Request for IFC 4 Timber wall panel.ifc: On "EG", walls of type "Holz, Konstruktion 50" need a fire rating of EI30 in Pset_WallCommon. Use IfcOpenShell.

First a look at what the model holds.

```python
import ifcopenshell
import ifcopenshell.util.element

model = ifcopenshell.open("IFC 4 Timber wall panel.ifc")
print(model.schema)
storey = next(s for s in model.by_type("IfcBuildingStorey") if s.Name == "EG")
walls = [e for e in ifcopenshell.util.element.get_decomposition(storey) if e.is_a("IfcWall")]
seen = {}
for e in walls:
    element_type = ifcopenshell.util.element.get_type(e)
    key = (element_type.Name if element_type != e and element_type else None, ifcopenshell.util.element.get_pset(e, "Pset_WallCommon", "FireRating"))
    seen[key] = seen.get(key, 0) + 1
for (name, value), count in sorted(seen.items(), key=str):
    print(count, "x", name, "|", value)
```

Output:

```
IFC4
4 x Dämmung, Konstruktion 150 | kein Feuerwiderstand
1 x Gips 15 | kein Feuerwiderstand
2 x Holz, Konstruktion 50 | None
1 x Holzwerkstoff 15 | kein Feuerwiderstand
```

```python
import ifcopenshell
import ifcopenshell.api.pset
import ifcopenshell.util.element

model = ifcopenshell.open("IFC 4 Timber wall panel.ifc")

storey = next(s for s in model.by_type("IfcBuildingStorey") if s.Name == "EG")
walls = [e for e in ifcopenshell.util.element.get_decomposition(storey) if e.is_a("IfcWall")]

count = 0
for e in walls:
    element_type = ifcopenshell.util.element.get_type(e)
    if element_type in (None, e) or element_type.Name != "Holz, Konstruktion 50":
        continue
    # add_pset returns the element's existing set when there is one.
    pset = ifcopenshell.api.pset.add_pset(model, product=e, name="Pset_WallCommon")
    ifcopenshell.api.pset.edit_pset(model, pset=pset, properties={"FireRating": "EI30"})
    count += 1

print(count, "walls updated")

model.write("IFC 4 Timber wall panel_updated.ifc")
```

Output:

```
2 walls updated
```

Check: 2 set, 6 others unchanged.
